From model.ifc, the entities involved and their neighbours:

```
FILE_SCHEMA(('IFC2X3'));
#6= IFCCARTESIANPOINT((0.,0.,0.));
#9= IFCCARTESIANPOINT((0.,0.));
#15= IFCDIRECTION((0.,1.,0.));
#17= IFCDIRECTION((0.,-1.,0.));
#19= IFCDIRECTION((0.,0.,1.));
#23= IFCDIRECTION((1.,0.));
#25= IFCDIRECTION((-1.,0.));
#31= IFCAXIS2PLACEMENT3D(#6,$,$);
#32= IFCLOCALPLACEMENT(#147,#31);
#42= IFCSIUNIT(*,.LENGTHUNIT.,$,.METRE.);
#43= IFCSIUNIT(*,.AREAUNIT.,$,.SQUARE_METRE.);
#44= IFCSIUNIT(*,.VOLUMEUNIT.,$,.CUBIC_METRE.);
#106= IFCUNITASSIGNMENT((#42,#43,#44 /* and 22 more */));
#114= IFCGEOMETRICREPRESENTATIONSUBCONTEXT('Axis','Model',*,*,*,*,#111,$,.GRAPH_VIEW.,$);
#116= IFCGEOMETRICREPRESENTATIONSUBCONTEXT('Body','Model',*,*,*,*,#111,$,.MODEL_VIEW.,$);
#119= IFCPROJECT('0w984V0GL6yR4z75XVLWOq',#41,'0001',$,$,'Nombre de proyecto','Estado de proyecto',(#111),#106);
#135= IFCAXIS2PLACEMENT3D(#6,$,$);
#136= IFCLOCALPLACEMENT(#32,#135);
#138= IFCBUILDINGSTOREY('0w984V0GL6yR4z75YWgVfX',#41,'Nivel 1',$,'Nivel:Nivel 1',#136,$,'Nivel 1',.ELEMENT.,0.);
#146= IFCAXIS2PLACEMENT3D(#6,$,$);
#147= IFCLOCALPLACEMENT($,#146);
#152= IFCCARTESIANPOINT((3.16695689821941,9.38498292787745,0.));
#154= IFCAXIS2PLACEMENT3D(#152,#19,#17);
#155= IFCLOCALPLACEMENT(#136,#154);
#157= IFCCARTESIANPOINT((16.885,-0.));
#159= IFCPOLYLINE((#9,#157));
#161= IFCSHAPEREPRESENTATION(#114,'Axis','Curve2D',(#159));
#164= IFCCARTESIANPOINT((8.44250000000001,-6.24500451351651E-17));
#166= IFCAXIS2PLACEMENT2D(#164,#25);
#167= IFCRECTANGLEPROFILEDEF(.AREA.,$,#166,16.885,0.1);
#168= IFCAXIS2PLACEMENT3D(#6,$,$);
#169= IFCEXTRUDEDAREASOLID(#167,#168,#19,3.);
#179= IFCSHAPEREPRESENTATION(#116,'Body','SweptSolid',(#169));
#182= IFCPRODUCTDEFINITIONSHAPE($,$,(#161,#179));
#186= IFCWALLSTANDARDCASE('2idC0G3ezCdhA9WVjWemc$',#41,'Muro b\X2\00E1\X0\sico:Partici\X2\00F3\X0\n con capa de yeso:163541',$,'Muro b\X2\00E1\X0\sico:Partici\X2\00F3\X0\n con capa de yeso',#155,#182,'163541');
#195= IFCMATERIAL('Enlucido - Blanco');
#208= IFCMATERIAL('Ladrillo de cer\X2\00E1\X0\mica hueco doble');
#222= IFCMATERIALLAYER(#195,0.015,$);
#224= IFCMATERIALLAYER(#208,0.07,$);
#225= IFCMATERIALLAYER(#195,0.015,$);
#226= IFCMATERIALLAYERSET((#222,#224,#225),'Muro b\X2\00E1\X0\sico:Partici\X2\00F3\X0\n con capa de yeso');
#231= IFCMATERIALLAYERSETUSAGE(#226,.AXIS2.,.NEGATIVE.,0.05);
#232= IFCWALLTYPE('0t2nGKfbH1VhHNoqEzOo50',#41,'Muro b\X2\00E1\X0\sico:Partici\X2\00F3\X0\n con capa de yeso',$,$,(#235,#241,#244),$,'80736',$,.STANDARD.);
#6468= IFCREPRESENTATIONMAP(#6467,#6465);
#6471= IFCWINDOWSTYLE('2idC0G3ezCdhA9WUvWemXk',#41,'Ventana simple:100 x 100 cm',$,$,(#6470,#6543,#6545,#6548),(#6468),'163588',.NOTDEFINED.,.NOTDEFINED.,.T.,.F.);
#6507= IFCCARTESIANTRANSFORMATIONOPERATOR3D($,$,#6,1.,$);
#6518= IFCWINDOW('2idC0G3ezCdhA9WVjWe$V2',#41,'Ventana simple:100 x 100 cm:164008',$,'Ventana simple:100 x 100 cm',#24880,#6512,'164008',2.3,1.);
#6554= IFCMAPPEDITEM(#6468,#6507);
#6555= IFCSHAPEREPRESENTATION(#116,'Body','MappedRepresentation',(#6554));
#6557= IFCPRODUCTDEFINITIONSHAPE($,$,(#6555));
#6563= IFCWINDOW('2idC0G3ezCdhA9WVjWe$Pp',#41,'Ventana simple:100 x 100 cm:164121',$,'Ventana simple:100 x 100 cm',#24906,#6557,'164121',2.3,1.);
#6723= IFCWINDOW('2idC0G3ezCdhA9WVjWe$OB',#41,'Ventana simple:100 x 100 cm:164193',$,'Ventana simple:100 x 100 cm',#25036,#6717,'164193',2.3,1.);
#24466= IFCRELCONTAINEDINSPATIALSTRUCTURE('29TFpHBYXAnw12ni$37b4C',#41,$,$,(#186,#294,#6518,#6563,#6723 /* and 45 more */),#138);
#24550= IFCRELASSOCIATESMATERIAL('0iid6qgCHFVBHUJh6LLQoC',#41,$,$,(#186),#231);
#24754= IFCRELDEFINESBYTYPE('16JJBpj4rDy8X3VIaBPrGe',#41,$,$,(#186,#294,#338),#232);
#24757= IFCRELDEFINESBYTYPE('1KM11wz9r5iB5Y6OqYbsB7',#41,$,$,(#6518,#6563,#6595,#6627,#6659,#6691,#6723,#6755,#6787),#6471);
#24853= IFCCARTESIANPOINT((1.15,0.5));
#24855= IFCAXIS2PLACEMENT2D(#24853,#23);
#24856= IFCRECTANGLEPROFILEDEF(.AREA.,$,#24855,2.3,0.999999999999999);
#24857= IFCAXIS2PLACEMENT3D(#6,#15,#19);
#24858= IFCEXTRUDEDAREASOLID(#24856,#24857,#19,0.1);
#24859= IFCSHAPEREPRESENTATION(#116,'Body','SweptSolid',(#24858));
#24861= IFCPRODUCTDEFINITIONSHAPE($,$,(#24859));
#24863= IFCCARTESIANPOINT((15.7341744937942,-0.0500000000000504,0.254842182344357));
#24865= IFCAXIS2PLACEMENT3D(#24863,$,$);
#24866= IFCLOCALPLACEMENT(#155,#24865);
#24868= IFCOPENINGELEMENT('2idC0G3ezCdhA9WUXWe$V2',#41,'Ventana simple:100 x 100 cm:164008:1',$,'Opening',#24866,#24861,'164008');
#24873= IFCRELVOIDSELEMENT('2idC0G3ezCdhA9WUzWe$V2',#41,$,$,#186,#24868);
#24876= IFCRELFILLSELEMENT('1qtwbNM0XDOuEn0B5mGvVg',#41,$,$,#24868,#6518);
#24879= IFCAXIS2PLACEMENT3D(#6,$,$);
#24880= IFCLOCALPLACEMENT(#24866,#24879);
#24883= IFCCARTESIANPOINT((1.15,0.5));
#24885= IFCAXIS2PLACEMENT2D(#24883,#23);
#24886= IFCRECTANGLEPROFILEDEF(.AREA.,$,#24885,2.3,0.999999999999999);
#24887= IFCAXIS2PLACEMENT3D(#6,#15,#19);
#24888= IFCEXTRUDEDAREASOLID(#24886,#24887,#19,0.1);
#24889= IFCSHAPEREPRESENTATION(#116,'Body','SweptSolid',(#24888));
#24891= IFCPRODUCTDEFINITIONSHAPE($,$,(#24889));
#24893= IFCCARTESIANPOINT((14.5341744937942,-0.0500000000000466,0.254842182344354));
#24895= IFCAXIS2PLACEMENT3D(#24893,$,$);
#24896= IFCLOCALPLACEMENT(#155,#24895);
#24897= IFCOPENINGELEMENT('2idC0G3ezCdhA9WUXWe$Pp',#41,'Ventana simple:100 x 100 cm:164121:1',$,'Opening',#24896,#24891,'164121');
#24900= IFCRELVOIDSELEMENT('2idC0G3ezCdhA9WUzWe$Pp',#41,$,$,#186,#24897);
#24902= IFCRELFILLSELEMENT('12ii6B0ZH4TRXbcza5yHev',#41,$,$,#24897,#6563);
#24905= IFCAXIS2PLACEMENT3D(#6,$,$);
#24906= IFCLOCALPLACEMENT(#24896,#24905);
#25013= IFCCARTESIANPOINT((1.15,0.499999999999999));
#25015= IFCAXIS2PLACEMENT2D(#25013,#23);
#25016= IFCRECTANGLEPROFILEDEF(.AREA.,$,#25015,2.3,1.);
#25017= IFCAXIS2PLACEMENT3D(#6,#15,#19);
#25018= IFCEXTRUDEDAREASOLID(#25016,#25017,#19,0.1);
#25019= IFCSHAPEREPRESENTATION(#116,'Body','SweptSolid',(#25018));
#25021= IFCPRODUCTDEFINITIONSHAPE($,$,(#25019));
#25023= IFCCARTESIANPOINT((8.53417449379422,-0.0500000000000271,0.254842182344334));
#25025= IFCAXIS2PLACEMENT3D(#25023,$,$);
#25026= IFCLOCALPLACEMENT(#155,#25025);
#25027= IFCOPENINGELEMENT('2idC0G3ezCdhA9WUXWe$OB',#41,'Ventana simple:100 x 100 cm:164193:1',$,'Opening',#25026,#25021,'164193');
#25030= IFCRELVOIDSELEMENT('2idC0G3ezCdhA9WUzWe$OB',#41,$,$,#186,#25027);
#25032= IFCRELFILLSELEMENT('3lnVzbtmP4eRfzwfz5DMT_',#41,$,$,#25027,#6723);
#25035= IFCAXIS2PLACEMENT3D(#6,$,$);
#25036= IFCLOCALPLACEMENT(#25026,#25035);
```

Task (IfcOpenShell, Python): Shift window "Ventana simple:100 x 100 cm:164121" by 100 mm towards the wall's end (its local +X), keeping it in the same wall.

```python
import ifcopenshell
import ifcopenshell.api.geometry
import ifcopenshell.util.placement
import ifcopenshell.util.unit

model = ifcopenshell.open("model.ifc")
unit_scale = ifcopenshell.util.unit.calculate_unit_scale(model)

window = model.by_id(6563)
opening = window.FillsVoids[0].RelatingOpeningElement
wall = opening.VoidsElements[0].RelatingBuildingElement

wall_matrix = ifcopenshell.util.placement.get_local_placement(wall.ObjectPlacement)
shift = wall_matrix[:3, 0] * 0.1 / unit_scale
before = ifcopenshell.util.placement.get_local_placement(window.ObjectPlacement)[:3, 3].copy()

# The window is placed relative to its opening, so it follows when the opening moves.
matrix = ifcopenshell.util.placement.get_local_placement(opening.ObjectPlacement)
matrix[:3, 3] += shift
ifcopenshell.api.geometry.edit_object_placement(
    model, product=opening, matrix=matrix, is_si=False, should_transform_children=True
)

after = ifcopenshell.util.placement.get_local_placement(window.ObjectPlacement)[:3, 3]
print("window moved by", (after - before).round(3) + 0.0)

model.write("model_rev.ifc")
```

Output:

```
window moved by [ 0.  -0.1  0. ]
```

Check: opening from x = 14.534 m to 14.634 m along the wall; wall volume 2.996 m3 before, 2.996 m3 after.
